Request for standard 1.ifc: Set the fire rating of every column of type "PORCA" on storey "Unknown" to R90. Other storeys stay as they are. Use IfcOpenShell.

First a look at what the model holds.

```python
import ifcopenshell
import ifcopenshell.util.element

model = ifcopenshell.open("standard 1.ifc")
print(model.schema)
storey = next(s for s in model.by_type("IfcBuildingStorey") if s.Name == "Unknown")
columns = [e for e in ifcopenshell.util.element.get_decomposition(storey) if e.is_a("IfcColumn")]
seen = {}
for e in columns:
    element_type = ifcopenshell.util.element.get_type(e)
    key = (element_type.Name if element_type != e and element_type else None, ifcopenshell.util.element.get_pset(e, "Pset_ColumnCommon", "FireRating"))
    seen[key] = seen.get(key, 0) + 1
for (name, value), count in sorted(seen.items(), key=str):
    print(count, "x", name, "|", value)
```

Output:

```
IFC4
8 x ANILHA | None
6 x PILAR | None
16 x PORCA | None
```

```python
import ifcopenshell
import ifcopenshell.api.pset
import ifcopenshell.util.element

model = ifcopenshell.open("standard 1.ifc")

storey = next(s for s in model.by_type("IfcBuildingStorey") if s.Name == "Unknown")
columns = [e for e in ifcopenshell.util.element.get_decomposition(storey) if e.is_a("IfcColumn")]

count = 0
for e in columns:
    element_type = ifcopenshell.util.element.get_type(e)
    if element_type in (None, e) or element_type.Name != "PORCA":
        continue
    found = ifcopenshell.util.element.get_pset(e, "Pset_ColumnCommon", should_inherit=False)
    if found:
        pset = model.by_id(found["id"])
        if len(ifcopenshell.util.element.get_elements_by_pset(pset)) > 1:
            pset = ifcopenshell.api.pset.unshare_pset(model, products=[e], pset=pset)[0]
    else:
        pset = ifcopenshell.api.pset.add_pset(model, product=e, name="Pset_ColumnCommon")
    ifcopenshell.api.pset.edit_pset(model, pset=pset, properties={"FireRating": "R90"})
    count += 1

print(count, "columns updated")

model.write("standard 1-out.ifc")
```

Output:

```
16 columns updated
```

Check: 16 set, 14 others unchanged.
